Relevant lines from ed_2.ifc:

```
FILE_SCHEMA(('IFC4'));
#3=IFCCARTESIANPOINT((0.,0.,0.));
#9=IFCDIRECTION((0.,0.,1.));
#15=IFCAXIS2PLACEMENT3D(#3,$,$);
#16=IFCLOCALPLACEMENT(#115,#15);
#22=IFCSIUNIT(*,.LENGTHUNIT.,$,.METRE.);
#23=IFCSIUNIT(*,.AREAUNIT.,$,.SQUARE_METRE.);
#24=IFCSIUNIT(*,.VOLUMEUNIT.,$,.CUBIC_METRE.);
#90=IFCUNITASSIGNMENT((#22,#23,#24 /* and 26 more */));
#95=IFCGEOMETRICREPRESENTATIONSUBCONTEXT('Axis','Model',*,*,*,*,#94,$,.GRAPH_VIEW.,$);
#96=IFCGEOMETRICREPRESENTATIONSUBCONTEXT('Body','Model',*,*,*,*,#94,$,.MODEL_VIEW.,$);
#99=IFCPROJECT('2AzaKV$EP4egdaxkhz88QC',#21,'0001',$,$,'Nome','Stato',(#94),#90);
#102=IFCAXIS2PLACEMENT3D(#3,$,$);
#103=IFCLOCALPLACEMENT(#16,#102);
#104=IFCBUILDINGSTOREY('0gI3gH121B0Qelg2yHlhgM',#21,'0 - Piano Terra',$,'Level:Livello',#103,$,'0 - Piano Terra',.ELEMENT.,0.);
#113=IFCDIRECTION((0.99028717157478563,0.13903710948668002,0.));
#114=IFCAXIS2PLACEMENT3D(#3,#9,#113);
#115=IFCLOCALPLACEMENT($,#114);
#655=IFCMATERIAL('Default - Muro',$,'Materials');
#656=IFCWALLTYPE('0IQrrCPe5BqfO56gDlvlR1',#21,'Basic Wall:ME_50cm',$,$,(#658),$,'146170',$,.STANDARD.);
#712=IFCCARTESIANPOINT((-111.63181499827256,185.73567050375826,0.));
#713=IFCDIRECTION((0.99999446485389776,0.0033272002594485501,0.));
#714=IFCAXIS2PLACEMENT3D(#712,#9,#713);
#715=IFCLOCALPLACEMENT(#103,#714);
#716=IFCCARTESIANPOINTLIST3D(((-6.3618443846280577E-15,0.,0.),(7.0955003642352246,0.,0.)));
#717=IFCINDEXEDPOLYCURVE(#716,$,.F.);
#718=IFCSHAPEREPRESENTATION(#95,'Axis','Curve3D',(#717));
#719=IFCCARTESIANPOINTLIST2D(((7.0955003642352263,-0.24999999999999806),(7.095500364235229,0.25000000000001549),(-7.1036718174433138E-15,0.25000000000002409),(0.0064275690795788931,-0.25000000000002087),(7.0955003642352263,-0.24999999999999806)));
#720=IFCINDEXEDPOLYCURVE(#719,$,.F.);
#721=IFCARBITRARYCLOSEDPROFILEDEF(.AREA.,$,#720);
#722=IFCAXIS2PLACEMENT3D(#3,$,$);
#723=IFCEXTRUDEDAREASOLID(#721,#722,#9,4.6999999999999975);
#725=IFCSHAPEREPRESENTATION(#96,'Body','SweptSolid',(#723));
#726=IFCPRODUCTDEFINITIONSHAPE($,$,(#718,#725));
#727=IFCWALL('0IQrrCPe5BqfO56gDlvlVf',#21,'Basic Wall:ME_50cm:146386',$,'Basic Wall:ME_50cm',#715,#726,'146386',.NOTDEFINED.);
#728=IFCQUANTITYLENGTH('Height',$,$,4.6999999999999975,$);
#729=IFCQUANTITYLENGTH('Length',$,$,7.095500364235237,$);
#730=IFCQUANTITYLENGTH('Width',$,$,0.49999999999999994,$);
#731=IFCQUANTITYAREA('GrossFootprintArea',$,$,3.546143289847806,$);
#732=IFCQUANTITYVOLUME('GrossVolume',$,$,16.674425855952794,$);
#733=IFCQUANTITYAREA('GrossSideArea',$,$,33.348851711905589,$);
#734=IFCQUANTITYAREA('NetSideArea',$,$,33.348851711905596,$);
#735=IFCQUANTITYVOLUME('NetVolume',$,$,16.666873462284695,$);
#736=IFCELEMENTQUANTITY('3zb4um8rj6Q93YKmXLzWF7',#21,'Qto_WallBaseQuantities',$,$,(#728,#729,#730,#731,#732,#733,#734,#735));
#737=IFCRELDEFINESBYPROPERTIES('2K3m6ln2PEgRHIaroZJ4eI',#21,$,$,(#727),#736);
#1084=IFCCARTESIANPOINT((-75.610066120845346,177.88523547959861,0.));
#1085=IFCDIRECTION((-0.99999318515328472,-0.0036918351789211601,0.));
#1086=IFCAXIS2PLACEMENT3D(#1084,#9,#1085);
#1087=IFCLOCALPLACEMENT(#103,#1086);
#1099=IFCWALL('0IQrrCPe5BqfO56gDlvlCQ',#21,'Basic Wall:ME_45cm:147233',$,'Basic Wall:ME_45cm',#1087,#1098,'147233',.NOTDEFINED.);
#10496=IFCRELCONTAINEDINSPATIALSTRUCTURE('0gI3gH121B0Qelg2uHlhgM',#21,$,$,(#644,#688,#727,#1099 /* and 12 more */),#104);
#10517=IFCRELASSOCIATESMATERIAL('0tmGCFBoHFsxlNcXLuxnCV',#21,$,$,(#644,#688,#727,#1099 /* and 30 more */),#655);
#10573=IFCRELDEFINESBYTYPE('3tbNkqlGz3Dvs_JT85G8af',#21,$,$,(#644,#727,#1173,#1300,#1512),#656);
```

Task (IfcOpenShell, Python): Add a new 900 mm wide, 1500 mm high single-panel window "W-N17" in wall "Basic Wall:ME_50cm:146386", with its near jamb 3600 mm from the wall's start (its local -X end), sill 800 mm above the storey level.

```python
import numpy as np
import ifcopenshell
import ifcopenshell.api.feature
import ifcopenshell.api.geometry
import ifcopenshell.api.pset
import ifcopenshell.api.root
import ifcopenshell.api.spatial
import ifcopenshell.geom
import ifcopenshell.util.element
import ifcopenshell.util.placement
import ifcopenshell.util.representation
import ifcopenshell.util.shape
import ifcopenshell.util.unit

model = ifcopenshell.open("ed_2.ifc")
unit_scale = ifcopenshell.util.unit.calculate_unit_scale(model)
area_scale = ifcopenshell.util.unit.calculate_unit_scale(model, "AREAUNIT")
volume_scale = ifcopenshell.util.unit.calculate_unit_scale(model, "VOLUMEUNIT")
settings = ifcopenshell.geom.settings()


def volume(element):
    """Net volume in cubic metres, openings subtracted."""
    shape = ifcopenshell.geom.create_shape(settings, element)
    return ifcopenshell.util.shape.get_volume(shape.geometry)


wall = model.by_id(727)
storey = ifcopenshell.util.element.get_container(wall, ifc_class="IfcBuildingStorey")
context = ifcopenshell.util.representation.get_context(model, "Model", "Body", "MODEL_VIEW")
before = volume(wall)

width, height, from_end, sill = 0.9, 1.5, 3.6, 0.8  # metres

# The wall runs along its own X axis, and the end named is its -X end.
wall_shape = ifcopenshell.geom.create_shape(settings, wall)
x, y, z = ifcopenshell.util.shape.get_vertices(wall_shape.geometry).T
start = x.min() + from_end
face, thickness = float(y.min()), float(y.max() - y.min())
wall_matrix = ifcopenshell.util.placement.get_local_placement(wall.ObjectPlacement)
level = ifcopenshell.util.placement.get_local_placement(storey.ObjectPlacement)[2, 3]


def in_wall(x, y):
    """Placement at x, y metres in the wall's axes, at sill height."""
    matrix = wall_matrix.copy()
    matrix[:, 3] = wall_matrix @ np.array([x / unit_scale, y / unit_scale, 0.0, 1.0])
    matrix[2, 3] = level + sill / unit_scale
    return matrix


# Opening: a box that overshoots both wall faces by 50 mm.
opening = ifcopenshell.api.root.create_entity(model, ifc_class="IfcOpeningElement", predefined_type="OPENING")
box = ifcopenshell.api.geometry.add_wall_representation(
    model, context=context, length=width, height=height, thickness=thickness + 0.1
)
ifcopenshell.api.geometry.assign_representation(model, product=opening, representation=box)
ifcopenshell.api.geometry.edit_object_placement(model, product=opening, matrix=in_wall(start, face - 0.05), is_si=False)
ifcopenshell.api.feature.add_feature(model, feature=opening, element=wall)

window = ifcopenshell.api.root.create_entity(model, ifc_class="IfcWindow", name="W-N17", predefined_type="WINDOW")
window.OverallWidth, window.OverallHeight = width / unit_scale, height / unit_scale
window.PartitioningType = "SINGLE_PANEL"
body = ifcopenshell.api.geometry.add_window_representation(
    model,
    context=context,
    overall_width=window.OverallWidth,
    overall_height=window.OverallHeight,
    partition_type="SINGLE_PANEL",
)
ifcopenshell.api.geometry.assign_representation(model, product=window, representation=body)
ifcopenshell.api.spatial.assign_container(model, products=[window], relating_structure=storey)
ifcopenshell.api.feature.add_filling(model, opening=opening, element=window)

# Centre the window in the wall's thickness.
ifcopenshell.api.geometry.edit_object_placement(model, product=window, matrix=in_wall(start, face), is_si=False)
window_shape = ifcopenshell.geom.create_shape(settings, window)
depth = ifcopenshell.util.shape.get_vertices(window_shape.geometry)[:, 1]
offset = face + thickness / 2 - (depth.min() + depth.max()) / 2
ifcopenshell.api.geometry.edit_object_placement(model, product=window, matrix=in_wall(start, offset), is_si=False)

after = volume(wall)

# Update the wall's stored quantities.
qto = model.by_id(ifcopenshell.util.element.get_pset(wall, "Qto_WallBaseQuantities", should_inherit=False)["id"])
ifcopenshell.api.pset.edit_qto(model, qto=qto, properties={
    "NetSideArea": after / thickness / area_scale,
    "NetVolume": after / volume_scale,
})

print(f"wall volume {before:.3f} -> {after:.3f} m3")

model.write("ed_2_v2.ifc")
```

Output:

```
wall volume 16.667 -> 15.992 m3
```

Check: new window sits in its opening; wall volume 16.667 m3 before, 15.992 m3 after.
